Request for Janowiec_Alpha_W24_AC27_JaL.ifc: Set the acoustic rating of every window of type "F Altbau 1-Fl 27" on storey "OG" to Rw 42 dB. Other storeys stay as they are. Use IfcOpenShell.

First a look at what the model holds.

```python
import ifcopenshell
import ifcopenshell.util.element

model = ifcopenshell.open("Janowiec_Alpha_W24_AC27_JaL.ifc")
print(model.schema)
storey = next(s for s in model.by_type("IfcBuildingStorey") if s.Name == "OG")
windows = [e for e in ifcopenshell.util.element.get_decomposition(storey) if e.is_a("IfcWindow")]
seen = {}
for e in windows:
    element_type = ifcopenshell.util.element.get_type(e)
    key = (element_type.Name if element_type != e and element_type else None, ifcopenshell.util.element.get_pset(e, "Pset_WindowCommon", "AcousticRating"))
    seen[key] = seen.get(key, 0) + 1
for (name, value), count in sorted(seen.items(), key=str):
    print(count, "x", name, "|", value)
```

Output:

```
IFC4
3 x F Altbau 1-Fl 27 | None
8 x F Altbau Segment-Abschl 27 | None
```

```python
import ifcopenshell
import ifcopenshell.api.pset
import ifcopenshell.util.element

model = ifcopenshell.open("Janowiec_Alpha_W24_AC27_JaL.ifc")

storey = next(s for s in model.by_type("IfcBuildingStorey") if s.Name == "OG")
windows = [e for e in ifcopenshell.util.element.get_decomposition(storey) if e.is_a("IfcWindow")]

count = 0
for e in windows:
    element_type = ifcopenshell.util.element.get_type(e)
    if element_type in (None, e) or element_type.Name != "F Altbau 1-Fl 27":
        continue
    # add_pset returns the element's existing set when there is one.
    pset = ifcopenshell.api.pset.add_pset(model, product=e, name="Pset_WindowCommon")
    ifcopenshell.api.pset.edit_pset(model, pset=pset, properties={"AcousticRating": "Rw 42 dB"})
    count += 1

print(count, "windows updated")

model.write("Janowiec_Alpha_W24_AC27_JaL-out.ifc")
```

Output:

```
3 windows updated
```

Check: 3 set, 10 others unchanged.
